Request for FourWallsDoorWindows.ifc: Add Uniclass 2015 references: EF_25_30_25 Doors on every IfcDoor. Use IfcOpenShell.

First a look at what the model holds.

```python
import ifcopenshell

model = ifcopenshell.open("FourWallsDoorWindows.ifc")
print(model.schema)
print("classifications:", [c.Name for c in model.by_type("IfcClassification")])
for ifc_class in ("IfcDoor", "IfcRoof", "IfcStair", "IfcWall", "IfcWindow"):
    print(ifc_class, len(model.by_type(ifc_class)))
```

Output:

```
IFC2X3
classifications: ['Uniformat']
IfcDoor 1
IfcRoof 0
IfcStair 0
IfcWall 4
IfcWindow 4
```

```python
import ifcopenshell
import ifcopenshell.api.classification

model = ifcopenshell.open("FourWallsDoorWindows.ifc")

# IFC2X3 requires Source and Edition and has no link from the project to the system.
system = model.create_entity("IfcClassification", Source="NBS", Edition="2015", Name="Uniclass 2015")

codes = {
    "IfcDoor": ("EF_25_30_25", "Doors"),
}
for ifc_class, (code, name) in codes.items():
    products = model.by_type(ifc_class)
    ifcopenshell.api.classification.add_reference(
        model, products=products, classification=system, identification=code, name=name
    )
    print(code, len(products))

model.write("FourWallsDoorWindows_rev.ifc")
```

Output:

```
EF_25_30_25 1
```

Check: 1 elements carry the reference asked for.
